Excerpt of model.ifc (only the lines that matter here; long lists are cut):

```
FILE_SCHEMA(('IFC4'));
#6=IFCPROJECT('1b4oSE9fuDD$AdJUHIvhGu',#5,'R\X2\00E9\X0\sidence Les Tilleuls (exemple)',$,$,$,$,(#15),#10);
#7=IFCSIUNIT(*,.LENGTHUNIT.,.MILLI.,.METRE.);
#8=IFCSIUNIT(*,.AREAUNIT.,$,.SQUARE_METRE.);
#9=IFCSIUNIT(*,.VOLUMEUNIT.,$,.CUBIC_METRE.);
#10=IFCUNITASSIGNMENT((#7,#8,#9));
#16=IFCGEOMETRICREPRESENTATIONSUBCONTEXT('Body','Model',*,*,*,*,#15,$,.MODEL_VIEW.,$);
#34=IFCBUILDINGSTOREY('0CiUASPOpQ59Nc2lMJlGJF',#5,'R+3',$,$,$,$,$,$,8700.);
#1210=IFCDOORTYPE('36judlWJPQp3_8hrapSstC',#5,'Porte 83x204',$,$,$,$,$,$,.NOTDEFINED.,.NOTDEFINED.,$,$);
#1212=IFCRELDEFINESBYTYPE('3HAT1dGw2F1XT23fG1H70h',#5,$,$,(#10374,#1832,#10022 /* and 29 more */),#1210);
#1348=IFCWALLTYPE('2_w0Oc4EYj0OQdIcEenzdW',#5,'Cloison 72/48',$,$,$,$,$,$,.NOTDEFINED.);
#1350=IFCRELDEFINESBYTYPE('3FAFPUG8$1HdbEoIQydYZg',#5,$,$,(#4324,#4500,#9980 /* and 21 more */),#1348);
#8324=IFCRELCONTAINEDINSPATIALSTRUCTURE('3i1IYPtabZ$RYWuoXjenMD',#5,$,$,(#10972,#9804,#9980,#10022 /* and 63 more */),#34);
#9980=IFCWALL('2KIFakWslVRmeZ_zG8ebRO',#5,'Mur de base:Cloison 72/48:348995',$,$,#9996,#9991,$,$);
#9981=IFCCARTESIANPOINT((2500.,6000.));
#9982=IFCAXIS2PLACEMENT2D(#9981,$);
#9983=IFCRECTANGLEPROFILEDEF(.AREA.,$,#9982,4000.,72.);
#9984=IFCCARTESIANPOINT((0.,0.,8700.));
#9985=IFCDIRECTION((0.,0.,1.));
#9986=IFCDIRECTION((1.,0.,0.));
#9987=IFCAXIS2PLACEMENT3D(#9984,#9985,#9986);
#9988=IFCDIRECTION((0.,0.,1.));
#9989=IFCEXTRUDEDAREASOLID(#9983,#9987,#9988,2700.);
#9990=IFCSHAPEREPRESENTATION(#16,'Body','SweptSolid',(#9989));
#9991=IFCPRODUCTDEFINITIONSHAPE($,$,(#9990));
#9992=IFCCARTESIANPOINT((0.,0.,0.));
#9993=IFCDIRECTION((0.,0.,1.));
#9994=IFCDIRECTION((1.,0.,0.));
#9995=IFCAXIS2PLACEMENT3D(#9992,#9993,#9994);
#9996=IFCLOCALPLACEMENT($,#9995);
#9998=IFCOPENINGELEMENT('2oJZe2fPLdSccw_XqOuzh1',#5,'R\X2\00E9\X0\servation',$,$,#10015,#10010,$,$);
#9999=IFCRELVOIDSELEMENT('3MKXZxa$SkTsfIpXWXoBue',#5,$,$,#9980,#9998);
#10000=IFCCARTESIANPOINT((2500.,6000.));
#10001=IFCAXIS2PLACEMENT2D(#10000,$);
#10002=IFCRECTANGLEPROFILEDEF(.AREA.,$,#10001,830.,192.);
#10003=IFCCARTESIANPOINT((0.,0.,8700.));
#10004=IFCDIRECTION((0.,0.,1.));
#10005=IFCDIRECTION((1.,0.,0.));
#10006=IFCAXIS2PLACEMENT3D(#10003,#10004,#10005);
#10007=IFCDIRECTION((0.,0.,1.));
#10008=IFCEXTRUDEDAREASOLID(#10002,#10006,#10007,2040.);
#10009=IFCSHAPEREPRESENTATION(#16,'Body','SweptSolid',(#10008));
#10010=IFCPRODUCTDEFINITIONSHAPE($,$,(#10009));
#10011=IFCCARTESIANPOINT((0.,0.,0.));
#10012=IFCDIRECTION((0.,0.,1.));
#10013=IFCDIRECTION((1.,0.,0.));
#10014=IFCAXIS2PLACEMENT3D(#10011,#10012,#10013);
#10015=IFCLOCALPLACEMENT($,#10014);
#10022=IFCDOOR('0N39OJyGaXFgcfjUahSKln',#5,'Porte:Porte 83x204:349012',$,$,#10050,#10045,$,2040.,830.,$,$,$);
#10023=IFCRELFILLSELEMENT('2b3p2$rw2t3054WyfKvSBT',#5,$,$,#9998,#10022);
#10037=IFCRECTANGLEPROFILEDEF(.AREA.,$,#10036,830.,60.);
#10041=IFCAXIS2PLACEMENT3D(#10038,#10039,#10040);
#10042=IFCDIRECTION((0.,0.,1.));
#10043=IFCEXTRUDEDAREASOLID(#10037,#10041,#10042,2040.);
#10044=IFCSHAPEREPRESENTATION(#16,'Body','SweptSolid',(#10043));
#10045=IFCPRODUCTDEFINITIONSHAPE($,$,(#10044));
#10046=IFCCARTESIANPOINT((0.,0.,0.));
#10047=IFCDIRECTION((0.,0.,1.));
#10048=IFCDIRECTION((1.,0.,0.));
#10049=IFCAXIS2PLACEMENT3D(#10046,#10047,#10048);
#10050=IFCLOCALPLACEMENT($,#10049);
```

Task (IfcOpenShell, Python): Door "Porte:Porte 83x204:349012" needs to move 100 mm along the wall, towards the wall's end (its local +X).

```python
import ifcopenshell
import ifcopenshell.api.geometry
import ifcopenshell.util.placement

model = ifcopenshell.open("model.ifc")

door = model.by_id(10022)
opening = door.FillsVoids[0].RelatingOpeningElement
wall = opening.VoidsElements[0].RelatingBuildingElement

wall_matrix = ifcopenshell.util.placement.get_local_placement(wall.ObjectPlacement)
shift = wall_matrix[:3, 0] * 100.0
before = ifcopenshell.util.placement.get_local_placement(door.ObjectPlacement)[:3, 3].copy()

# The door is not placed relative to its opening, so move both.
for product in (opening, door):
    matrix = ifcopenshell.util.placement.get_local_placement(product.ObjectPlacement)
    matrix[:3, 3] += shift
    ifcopenshell.api.geometry.edit_object_placement(model, product=product, matrix=matrix, is_si=False)

after = ifcopenshell.util.placement.get_local_placement(door.ObjectPlacement)[:3, 3]
print("door moved by", (after - before).round(3) + 0.0)

model.write("model_rev.ifc")
```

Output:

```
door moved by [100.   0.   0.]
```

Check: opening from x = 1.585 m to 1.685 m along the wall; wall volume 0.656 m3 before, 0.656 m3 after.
